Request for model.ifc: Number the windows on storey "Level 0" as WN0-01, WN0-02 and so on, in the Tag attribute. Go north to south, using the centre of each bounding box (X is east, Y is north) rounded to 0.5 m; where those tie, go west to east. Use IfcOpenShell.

First a look at what the model holds.

```python
import ifcopenshell
import ifcopenshell.util.element
import ifcopenshell.util.placement

model = ifcopenshell.open("model.ifc")
print(model.schema)
storey = next(s for s in model.by_type("IfcBuildingStorey") if s.Name == "Level 0")
windows = [e for e in ifcopenshell.util.element.get_decomposition(storey) if e.is_a("IfcWindow")]
for e in sorted(windows, key=lambda e: e.id()):
    origin = ifcopenshell.util.placement.get_local_placement(e.ObjectPlacement)[:3, 3]
    print(e.id(), e.Tag, e.Name, origin.round(2) + 0.0, sep=" | ")
```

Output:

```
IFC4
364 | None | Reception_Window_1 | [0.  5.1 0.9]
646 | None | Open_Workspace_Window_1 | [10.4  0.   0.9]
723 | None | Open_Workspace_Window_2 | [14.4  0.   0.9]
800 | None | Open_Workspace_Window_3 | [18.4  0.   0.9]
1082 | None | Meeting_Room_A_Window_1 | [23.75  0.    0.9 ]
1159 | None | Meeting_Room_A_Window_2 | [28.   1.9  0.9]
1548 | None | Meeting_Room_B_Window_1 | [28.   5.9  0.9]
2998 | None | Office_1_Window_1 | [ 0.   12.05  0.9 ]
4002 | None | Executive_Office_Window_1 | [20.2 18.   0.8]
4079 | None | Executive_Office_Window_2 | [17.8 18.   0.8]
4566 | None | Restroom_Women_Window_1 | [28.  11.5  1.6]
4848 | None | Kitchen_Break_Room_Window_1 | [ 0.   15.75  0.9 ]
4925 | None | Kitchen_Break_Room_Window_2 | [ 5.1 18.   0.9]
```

```python
import ifcopenshell
import ifcopenshell.geom
import ifcopenshell.util.element
import ifcopenshell.util.shape

model = ifcopenshell.open("model.ifc")
settings = ifcopenshell.geom.settings()
settings.set("use-world-coords", True)


def centre(element):
    shape = ifcopenshell.geom.create_shape(settings, element)
    return ifcopenshell.util.shape.get_bbox_centroid(shape.geometry)


storey = next(s for s in model.by_type("IfcBuildingStorey") if s.Name == "Level 0")
windows = [e for e in ifcopenshell.util.element.get_decomposition(storey) if e.is_a("IfcWindow")]

# Insertion points can sit at a corner or the storey origin, so sort by the geometry (in metres).
centres = {e: centre(e) for e in windows}
windows.sort(key=lambda e: (-round(centres[e][1] / 0.5), centres[e][0]))

for i, e in enumerate(windows, start=1):
    number = f"WN0-{i:02d}"
    e.Tag = number
    print(e.id(), number)

model.write("model_updated.ifc")
```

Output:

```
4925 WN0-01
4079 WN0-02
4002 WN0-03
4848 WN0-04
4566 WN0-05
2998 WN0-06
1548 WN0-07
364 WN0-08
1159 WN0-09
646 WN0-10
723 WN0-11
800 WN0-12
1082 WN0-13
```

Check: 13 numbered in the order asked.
